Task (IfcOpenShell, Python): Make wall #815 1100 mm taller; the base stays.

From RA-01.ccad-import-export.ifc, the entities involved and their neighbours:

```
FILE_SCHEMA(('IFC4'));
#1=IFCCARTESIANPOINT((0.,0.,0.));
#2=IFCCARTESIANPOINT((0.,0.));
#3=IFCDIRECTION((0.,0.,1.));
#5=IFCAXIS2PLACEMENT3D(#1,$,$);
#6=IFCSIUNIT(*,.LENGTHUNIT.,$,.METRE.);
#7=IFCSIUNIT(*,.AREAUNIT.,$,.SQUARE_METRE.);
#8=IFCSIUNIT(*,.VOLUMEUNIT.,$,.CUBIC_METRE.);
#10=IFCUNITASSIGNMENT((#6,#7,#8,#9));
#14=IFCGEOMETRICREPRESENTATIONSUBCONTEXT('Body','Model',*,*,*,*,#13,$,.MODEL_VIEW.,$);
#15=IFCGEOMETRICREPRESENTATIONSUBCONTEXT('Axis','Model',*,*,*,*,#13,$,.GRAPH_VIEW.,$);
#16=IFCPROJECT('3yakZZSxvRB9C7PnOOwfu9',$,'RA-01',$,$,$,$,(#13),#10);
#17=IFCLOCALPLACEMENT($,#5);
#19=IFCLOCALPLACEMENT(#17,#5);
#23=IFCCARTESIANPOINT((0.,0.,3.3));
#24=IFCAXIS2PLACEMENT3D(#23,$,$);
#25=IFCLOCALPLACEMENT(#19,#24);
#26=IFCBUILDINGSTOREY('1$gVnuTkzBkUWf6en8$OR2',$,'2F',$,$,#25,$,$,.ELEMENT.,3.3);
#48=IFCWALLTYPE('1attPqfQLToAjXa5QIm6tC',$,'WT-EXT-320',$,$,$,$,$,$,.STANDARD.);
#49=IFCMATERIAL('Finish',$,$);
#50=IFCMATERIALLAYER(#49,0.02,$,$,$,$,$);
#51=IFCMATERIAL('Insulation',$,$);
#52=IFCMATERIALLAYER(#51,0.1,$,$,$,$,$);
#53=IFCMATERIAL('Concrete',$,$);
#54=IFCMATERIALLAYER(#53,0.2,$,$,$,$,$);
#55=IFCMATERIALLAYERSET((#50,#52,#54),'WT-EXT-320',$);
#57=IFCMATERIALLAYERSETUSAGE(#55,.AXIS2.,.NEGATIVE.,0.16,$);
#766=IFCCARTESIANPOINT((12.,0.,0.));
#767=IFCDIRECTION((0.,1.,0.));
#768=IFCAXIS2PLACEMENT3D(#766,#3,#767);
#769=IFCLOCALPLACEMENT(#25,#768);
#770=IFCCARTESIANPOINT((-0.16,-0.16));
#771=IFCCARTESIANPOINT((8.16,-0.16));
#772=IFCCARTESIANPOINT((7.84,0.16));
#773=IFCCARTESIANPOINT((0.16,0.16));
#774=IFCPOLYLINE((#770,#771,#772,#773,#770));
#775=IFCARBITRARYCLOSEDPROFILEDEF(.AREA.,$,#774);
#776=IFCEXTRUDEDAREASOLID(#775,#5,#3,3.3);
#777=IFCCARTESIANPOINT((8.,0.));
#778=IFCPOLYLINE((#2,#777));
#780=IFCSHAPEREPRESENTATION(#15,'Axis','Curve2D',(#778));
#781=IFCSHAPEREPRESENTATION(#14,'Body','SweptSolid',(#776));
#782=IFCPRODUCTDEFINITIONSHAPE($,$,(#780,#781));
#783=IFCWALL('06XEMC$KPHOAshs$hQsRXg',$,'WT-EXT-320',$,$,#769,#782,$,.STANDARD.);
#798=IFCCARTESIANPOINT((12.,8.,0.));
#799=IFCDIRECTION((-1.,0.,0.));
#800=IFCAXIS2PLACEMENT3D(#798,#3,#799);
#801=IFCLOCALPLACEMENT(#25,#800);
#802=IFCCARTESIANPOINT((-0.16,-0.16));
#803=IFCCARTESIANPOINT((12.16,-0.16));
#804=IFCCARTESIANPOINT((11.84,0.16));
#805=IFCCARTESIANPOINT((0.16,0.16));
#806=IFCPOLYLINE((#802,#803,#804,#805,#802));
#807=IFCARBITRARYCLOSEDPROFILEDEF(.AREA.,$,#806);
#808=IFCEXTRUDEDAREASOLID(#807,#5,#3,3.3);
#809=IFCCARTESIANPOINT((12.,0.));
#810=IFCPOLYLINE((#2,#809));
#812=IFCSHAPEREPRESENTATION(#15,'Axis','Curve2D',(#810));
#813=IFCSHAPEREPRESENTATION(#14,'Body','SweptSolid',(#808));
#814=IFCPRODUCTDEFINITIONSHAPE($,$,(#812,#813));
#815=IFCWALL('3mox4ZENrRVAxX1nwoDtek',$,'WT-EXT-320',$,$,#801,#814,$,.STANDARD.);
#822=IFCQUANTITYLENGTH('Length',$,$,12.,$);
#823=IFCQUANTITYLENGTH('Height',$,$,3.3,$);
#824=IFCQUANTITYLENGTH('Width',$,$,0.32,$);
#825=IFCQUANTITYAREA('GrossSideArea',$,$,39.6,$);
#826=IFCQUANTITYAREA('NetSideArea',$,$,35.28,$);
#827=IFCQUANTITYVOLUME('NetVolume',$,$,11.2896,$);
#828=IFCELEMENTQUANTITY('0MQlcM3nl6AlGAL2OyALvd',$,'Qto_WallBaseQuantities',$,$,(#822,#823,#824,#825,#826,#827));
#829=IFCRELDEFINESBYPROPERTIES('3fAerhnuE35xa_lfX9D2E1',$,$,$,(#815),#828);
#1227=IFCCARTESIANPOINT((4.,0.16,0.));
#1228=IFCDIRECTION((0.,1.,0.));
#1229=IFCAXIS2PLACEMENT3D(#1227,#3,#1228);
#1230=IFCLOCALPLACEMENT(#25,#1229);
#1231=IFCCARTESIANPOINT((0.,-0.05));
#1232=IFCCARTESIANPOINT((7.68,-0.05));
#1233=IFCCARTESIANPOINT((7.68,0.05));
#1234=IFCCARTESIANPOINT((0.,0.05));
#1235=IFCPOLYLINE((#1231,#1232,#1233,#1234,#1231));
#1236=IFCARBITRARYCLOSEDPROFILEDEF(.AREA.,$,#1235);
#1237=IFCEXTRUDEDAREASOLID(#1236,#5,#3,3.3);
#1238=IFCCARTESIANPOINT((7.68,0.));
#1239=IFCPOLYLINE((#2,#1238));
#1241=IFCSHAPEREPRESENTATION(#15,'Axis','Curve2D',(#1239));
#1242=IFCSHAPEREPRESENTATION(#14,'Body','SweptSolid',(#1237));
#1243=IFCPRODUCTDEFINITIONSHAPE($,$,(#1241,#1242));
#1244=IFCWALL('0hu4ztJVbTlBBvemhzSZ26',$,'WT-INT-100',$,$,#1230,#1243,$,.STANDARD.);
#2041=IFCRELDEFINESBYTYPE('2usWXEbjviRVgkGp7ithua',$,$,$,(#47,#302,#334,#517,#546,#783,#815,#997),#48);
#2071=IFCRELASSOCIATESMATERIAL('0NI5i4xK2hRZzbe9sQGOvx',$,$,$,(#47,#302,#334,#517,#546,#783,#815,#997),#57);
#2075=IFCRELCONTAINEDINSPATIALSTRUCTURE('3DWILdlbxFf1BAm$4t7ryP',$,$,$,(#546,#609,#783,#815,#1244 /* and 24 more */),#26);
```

```python
import ifcopenshell
import ifcopenshell.api.pset
import ifcopenshell.geom
import ifcopenshell.util.element
import ifcopenshell.util.representation
import ifcopenshell.util.shape
import ifcopenshell.util.unit

model = ifcopenshell.open("RA-01.ccad-import-export.ifc")
unit_scale = ifcopenshell.util.unit.calculate_unit_scale(model)
area_scale = ifcopenshell.util.unit.calculate_unit_scale(model, "AREAUNIT")
volume_scale = ifcopenshell.util.unit.calculate_unit_scale(model, "VOLUMEUNIT")
settings = ifcopenshell.geom.settings()


def volume(element):
    """Net volume in cubic metres, openings subtracted."""
    shape = ifcopenshell.geom.create_shape(settings, element)
    return ifcopenshell.util.shape.get_volume(shape.geometry)


wall = model.by_id(815)
before = volume(wall)

body = ifcopenshell.util.representation.get_representation(wall, "Model", "Body")
solid = body.Items[0]
old_height = solid.Depth
solid.Depth += 1.1 / unit_scale
after = volume(wall)
thickness = 0.32  # wall thickness in metres

# Update the stored height, areas and volumes.
qto = model.by_id(ifcopenshell.util.element.get_pset(wall, "Qto_WallBaseQuantities", should_inherit=False)["id"])
ifcopenshell.api.pset.edit_qto(model, qto=qto, properties={
    "Height": solid.Depth,
    "GrossSideArea": ifcopenshell.util.element.get_pset(wall, "Qto_WallBaseQuantities", "GrossSideArea") * solid.Depth / old_height,
    "NetSideArea": after / thickness / area_scale,
    "NetVolume": after / volume_scale,
})

print(f"height {old_height:g} -> {solid.Depth:g}, volume {before:.3f} -> {after:.3f} m3")

model.write("RA-01.ccad-import-export-out.ifc")
```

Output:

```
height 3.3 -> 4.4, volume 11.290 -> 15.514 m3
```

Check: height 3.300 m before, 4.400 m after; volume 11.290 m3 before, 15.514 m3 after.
